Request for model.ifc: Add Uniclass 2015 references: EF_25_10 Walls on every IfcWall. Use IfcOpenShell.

First a look at what the model holds.

```python
import ifcopenshell

model = ifcopenshell.open("model.ifc")
print(model.schema)
print("classifications:", [c.Name for c in model.by_type("IfcClassification")])
for ifc_class in ("IfcDoor", "IfcRoof", "IfcStair", "IfcWall", "IfcWindow"):
    print(ifc_class, len(model.by_type(ifc_class)))
```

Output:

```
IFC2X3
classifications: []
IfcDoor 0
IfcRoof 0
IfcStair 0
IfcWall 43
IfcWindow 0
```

```python
import ifcopenshell
import ifcopenshell.api.classification

model = ifcopenshell.open("model.ifc")

# IFC2X3 requires Source and Edition and has no link from the project to the system.
system = model.create_entity("IfcClassification", Source="NBS", Edition="2015", Name="Uniclass 2015")

codes = {
    "IfcWall": ("EF_25_10", "Walls"),
}
for ifc_class, (code, name) in codes.items():
    products = model.by_type(ifc_class)
    ifcopenshell.api.classification.add_reference(
        model, products=products, classification=system, identification=code, name=name
    )
    print(code, len(products))

model.write("model_updated.ifc")
```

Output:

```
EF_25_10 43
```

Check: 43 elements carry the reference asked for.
